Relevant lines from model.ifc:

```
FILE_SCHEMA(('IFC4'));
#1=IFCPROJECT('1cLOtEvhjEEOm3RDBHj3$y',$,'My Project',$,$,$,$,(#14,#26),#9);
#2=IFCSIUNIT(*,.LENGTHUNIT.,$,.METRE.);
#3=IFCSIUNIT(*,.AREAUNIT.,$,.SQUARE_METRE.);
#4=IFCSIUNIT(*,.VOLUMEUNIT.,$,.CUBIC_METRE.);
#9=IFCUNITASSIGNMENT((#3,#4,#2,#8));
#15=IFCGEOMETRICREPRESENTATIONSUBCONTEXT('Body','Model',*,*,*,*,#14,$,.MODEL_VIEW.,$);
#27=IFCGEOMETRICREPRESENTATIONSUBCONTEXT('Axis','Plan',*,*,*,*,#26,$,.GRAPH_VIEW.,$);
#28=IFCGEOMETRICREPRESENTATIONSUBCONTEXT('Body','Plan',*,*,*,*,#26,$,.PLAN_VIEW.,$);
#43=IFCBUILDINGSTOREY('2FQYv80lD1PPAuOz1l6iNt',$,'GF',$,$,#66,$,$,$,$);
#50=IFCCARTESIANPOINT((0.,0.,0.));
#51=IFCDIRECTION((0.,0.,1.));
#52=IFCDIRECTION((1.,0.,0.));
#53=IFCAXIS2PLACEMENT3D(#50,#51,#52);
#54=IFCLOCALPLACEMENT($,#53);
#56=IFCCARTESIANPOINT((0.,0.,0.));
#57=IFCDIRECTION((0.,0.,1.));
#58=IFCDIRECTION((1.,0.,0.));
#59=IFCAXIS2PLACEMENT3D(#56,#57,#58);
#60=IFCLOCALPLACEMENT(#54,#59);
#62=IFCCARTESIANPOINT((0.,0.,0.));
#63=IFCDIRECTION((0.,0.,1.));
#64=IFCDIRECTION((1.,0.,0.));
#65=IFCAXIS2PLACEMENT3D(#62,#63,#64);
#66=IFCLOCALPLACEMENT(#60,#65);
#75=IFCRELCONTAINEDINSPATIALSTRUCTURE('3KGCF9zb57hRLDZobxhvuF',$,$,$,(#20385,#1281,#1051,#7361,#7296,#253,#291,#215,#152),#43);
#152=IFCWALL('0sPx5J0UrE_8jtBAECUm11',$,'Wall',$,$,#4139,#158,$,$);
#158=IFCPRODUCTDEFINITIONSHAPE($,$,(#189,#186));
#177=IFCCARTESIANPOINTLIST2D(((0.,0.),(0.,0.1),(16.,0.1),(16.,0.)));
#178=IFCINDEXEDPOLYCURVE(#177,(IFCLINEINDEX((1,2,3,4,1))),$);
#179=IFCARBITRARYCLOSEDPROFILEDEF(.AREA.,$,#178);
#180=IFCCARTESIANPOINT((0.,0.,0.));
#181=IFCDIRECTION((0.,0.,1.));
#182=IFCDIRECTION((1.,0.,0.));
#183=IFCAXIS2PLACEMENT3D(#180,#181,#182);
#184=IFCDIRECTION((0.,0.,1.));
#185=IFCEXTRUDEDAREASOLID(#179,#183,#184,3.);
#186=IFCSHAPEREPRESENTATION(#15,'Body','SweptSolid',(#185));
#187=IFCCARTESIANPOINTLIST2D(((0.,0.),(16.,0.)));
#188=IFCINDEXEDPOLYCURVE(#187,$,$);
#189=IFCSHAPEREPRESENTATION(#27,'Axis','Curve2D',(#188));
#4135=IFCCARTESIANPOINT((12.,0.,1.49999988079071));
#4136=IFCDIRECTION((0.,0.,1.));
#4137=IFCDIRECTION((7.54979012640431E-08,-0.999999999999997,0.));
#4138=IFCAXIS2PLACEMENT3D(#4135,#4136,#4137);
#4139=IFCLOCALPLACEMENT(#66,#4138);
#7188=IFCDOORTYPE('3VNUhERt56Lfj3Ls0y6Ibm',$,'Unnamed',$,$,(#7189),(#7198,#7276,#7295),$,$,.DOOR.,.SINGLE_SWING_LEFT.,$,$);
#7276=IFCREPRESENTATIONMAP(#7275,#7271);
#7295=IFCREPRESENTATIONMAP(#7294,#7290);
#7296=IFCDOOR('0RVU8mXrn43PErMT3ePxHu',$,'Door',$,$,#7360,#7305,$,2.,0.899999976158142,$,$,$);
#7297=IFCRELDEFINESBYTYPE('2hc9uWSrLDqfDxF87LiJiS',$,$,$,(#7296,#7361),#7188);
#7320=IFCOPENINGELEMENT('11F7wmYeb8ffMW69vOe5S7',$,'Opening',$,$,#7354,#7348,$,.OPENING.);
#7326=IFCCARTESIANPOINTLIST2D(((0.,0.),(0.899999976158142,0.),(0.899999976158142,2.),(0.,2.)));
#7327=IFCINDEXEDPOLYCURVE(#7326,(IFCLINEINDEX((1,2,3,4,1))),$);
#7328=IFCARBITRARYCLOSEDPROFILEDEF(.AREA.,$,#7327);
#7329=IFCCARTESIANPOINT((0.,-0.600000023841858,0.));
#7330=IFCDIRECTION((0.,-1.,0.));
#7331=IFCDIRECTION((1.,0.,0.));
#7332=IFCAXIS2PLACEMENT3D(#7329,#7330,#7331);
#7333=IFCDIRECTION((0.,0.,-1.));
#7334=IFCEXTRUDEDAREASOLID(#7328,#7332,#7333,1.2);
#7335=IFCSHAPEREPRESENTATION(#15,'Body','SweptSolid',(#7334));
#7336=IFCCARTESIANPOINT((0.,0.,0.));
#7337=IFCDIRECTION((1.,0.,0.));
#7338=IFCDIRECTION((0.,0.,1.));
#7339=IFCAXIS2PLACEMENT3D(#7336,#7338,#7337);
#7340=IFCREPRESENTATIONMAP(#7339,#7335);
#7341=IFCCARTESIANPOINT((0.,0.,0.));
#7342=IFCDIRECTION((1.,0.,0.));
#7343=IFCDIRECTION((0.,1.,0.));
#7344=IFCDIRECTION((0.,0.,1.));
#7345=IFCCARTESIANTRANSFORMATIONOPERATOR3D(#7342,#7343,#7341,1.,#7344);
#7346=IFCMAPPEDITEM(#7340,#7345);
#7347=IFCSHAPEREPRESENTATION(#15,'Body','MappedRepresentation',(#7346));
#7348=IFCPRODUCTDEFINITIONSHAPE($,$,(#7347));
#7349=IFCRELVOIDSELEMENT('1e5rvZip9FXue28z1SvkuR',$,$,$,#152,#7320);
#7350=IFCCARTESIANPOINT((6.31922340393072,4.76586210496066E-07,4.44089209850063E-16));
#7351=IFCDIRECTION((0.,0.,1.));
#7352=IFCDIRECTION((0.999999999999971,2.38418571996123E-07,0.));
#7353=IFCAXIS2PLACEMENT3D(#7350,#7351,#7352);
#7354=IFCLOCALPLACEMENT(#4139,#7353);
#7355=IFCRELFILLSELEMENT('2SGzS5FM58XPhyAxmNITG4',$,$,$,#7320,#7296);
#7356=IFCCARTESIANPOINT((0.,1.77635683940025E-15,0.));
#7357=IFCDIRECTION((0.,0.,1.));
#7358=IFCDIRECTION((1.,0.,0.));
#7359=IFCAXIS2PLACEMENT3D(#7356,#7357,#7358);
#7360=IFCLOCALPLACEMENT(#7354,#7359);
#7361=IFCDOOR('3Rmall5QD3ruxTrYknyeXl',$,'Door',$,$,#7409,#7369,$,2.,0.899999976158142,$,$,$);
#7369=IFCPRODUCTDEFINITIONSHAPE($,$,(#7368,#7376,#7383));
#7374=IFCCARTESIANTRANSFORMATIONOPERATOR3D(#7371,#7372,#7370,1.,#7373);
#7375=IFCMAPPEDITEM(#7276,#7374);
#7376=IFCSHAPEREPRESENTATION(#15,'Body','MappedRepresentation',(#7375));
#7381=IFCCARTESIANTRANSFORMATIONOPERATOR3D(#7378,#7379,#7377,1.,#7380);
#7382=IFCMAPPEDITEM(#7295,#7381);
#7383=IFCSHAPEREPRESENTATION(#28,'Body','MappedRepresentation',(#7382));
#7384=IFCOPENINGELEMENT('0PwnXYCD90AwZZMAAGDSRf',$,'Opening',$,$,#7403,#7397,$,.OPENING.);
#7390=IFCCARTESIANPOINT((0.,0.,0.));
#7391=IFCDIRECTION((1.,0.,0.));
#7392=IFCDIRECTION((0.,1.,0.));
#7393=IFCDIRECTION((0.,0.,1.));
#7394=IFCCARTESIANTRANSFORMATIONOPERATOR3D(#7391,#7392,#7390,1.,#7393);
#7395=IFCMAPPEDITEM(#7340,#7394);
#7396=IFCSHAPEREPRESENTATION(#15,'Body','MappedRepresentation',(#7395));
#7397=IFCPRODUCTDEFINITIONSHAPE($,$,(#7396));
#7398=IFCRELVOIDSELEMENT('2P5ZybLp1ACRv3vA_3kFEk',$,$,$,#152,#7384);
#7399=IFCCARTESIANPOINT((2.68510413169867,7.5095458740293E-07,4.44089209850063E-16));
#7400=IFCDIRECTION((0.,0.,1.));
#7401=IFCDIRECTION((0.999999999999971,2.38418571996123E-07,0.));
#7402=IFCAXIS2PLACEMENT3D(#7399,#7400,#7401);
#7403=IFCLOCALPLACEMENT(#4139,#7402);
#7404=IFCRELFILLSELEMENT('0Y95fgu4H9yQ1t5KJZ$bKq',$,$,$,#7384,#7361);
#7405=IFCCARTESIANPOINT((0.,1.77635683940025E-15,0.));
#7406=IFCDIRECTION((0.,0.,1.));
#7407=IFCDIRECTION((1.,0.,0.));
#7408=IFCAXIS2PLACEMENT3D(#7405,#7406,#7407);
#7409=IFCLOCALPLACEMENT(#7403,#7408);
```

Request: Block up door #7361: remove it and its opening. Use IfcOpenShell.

```python
import ifcopenshell
import ifcopenshell.api.feature
import ifcopenshell.api.root
import ifcopenshell.geom
import ifcopenshell.util.shape

model = ifcopenshell.open("model.ifc")
settings = ifcopenshell.geom.settings()


def volume(element):
    """Net volume in cubic metres, openings subtracted."""
    shape = ifcopenshell.geom.create_shape(settings, element)
    return ifcopenshell.util.shape.get_volume(shape.geometry)


door = model.by_guid("3Rmall5QD3ruxTrYknyeXl")
opening = door.FillsVoids[0].RelatingOpeningElement
wall = opening.VoidsElements[0].RelatingBuildingElement
before = volume(wall)

ifcopenshell.api.root.remove_product(model, product=door)
ifcopenshell.api.feature.remove_feature(model, feature=opening)

after = volume(wall)

print(f"wall volume {before:.3f} -> {after:.3f} m3")

model.write("model_v2.ifc")
```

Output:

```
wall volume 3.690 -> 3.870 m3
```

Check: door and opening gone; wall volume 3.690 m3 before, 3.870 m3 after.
